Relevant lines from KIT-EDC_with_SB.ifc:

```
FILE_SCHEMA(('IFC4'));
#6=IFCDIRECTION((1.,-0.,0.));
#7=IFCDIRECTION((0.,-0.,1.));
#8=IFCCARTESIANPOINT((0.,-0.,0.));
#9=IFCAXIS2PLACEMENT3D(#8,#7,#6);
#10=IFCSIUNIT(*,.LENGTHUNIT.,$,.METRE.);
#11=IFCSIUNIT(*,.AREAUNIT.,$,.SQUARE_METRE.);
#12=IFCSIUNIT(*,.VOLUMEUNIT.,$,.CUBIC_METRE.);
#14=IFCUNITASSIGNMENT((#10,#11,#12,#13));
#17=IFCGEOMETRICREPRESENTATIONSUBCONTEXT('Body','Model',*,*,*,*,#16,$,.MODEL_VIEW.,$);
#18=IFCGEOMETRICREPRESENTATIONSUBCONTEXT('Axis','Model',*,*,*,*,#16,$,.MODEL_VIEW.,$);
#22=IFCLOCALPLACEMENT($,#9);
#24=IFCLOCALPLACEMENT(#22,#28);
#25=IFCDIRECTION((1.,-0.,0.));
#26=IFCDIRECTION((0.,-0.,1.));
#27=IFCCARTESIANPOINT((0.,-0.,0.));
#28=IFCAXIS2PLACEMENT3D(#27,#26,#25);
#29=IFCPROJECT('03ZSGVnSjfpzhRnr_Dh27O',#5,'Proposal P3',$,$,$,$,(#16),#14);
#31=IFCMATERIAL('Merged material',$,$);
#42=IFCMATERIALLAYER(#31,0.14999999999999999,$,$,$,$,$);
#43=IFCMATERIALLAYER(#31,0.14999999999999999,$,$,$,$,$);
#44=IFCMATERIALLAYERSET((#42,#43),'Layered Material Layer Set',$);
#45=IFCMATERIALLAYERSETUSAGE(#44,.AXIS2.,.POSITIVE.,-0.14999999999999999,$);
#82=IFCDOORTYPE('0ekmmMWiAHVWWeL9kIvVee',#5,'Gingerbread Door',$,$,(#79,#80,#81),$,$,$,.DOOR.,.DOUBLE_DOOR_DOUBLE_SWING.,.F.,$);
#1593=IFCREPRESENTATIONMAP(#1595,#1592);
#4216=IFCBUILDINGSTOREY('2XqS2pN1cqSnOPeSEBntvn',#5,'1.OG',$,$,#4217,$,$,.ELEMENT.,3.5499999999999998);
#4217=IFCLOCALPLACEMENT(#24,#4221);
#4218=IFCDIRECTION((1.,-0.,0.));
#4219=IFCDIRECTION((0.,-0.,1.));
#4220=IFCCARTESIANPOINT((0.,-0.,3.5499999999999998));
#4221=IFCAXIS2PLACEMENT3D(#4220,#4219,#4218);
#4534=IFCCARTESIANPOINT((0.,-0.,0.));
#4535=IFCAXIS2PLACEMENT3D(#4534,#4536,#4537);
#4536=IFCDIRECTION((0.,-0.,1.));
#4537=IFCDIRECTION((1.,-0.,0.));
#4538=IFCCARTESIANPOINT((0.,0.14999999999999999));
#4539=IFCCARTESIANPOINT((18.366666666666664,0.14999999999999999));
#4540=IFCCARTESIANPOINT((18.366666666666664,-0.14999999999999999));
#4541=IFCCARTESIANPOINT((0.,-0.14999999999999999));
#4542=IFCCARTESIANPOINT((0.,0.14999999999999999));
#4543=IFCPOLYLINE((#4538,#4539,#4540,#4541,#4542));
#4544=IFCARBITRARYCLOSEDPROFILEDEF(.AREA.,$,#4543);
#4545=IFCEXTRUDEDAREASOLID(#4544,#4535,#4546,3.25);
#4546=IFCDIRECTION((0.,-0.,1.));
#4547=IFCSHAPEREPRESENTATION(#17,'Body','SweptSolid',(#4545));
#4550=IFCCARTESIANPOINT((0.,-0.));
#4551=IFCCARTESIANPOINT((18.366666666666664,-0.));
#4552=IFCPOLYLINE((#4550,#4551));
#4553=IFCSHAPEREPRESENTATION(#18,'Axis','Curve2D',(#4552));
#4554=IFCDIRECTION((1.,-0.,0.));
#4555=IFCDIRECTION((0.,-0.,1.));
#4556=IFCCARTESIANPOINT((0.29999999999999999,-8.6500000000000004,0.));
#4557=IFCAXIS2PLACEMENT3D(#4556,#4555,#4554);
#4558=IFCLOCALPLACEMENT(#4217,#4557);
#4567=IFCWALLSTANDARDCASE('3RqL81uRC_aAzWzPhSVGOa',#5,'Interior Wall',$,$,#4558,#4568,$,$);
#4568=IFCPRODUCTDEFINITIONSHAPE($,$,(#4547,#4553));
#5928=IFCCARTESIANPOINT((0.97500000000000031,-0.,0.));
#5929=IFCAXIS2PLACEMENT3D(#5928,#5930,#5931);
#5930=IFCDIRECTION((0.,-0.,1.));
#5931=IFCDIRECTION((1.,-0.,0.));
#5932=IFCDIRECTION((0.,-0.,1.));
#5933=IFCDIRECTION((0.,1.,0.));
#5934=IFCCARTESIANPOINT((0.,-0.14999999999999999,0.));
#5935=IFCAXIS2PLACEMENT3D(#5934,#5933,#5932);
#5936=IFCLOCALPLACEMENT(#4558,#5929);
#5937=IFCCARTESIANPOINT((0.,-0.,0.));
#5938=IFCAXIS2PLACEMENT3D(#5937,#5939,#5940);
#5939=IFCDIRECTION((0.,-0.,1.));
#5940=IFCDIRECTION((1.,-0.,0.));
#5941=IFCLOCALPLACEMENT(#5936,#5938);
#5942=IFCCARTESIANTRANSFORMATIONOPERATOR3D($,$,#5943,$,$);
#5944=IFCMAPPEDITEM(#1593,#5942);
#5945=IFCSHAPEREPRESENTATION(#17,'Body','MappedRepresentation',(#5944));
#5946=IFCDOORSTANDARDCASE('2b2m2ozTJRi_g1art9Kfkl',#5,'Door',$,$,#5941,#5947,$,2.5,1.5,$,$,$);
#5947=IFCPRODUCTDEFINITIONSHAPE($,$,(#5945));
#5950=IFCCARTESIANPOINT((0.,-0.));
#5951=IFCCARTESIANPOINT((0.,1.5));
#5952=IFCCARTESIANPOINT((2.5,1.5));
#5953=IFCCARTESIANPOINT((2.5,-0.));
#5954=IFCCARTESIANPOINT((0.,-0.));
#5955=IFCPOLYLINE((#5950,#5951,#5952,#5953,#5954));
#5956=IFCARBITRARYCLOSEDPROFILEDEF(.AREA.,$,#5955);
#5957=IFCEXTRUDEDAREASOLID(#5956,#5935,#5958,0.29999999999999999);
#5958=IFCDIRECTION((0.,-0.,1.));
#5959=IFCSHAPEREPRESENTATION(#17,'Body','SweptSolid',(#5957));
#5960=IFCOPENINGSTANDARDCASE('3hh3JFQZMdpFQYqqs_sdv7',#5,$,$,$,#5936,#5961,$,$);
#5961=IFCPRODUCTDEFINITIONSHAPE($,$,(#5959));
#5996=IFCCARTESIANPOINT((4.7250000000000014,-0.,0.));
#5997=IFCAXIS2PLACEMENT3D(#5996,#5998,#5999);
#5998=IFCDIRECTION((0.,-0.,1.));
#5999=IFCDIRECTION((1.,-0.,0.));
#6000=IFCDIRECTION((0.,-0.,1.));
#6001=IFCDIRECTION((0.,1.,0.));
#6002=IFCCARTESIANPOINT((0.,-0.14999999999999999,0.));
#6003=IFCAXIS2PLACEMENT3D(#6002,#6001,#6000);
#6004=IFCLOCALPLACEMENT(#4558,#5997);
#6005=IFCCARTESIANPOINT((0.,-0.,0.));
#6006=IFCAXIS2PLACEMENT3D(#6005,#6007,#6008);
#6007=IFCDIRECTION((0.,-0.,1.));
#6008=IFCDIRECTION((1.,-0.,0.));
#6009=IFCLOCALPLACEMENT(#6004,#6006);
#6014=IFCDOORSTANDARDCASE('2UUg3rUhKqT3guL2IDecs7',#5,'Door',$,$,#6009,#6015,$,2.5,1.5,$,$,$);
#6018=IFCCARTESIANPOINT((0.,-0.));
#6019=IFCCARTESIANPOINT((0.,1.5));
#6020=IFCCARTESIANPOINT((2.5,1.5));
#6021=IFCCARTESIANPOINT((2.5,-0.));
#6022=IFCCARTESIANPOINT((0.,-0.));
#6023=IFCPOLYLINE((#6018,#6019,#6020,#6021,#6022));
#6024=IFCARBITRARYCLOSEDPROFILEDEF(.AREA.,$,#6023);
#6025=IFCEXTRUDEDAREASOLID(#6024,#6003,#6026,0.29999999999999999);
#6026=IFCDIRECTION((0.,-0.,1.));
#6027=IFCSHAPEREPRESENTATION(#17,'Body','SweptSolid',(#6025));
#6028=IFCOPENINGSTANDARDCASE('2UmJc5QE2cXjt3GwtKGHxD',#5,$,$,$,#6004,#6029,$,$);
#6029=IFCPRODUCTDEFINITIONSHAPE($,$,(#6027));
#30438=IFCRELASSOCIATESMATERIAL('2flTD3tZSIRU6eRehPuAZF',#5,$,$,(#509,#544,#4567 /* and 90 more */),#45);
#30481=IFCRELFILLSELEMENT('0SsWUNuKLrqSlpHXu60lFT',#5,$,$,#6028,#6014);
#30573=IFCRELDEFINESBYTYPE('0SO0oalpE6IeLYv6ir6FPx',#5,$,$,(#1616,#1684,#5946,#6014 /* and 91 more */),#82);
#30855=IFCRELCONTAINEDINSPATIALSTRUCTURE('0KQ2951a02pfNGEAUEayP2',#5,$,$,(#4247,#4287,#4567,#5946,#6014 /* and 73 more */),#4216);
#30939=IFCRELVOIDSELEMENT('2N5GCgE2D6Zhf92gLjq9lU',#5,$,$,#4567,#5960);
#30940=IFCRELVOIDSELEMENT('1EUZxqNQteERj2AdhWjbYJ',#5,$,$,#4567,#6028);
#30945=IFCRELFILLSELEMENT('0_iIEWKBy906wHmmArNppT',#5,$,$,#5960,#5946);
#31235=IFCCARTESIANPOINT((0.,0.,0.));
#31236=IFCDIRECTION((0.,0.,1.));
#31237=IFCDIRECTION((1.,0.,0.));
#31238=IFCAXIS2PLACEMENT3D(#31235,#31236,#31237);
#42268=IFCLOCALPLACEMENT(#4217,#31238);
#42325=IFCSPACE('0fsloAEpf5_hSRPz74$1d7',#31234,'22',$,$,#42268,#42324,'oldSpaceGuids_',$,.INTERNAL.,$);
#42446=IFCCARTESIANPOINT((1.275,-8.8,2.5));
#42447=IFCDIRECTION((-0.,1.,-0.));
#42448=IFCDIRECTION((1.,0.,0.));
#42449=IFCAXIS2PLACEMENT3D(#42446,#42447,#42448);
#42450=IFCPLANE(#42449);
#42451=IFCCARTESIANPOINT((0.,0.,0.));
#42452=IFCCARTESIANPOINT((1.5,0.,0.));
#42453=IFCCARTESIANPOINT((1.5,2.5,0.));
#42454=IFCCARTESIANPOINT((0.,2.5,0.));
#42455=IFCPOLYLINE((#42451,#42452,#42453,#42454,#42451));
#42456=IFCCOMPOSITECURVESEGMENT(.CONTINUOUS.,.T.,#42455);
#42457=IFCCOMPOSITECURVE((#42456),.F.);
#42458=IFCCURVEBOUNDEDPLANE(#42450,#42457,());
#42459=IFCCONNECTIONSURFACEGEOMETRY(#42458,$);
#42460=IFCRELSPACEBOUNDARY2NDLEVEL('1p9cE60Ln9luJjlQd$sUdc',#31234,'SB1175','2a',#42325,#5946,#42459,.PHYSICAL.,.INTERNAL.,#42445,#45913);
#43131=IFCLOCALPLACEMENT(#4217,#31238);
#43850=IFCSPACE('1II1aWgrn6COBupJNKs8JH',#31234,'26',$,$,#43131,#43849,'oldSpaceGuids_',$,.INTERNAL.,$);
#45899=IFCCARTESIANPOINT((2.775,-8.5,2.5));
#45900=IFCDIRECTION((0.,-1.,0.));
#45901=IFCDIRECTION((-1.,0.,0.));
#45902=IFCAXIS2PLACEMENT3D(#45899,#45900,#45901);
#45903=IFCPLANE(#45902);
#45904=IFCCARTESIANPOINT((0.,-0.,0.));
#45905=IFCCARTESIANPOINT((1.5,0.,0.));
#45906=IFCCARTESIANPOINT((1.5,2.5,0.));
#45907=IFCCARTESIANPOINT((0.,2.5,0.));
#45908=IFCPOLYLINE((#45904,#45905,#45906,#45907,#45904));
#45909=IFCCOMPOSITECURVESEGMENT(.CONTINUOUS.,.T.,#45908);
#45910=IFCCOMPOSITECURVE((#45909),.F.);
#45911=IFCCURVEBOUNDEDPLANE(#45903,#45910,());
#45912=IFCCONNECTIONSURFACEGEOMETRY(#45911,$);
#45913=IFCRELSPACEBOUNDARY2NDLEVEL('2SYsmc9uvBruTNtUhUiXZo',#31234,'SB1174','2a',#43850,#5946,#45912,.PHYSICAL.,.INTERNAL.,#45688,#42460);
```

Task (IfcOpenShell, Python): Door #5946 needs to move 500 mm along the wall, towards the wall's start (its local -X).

```python
import numpy as np
import ifcopenshell
import ifcopenshell.api.geometry
import ifcopenshell.util.placement
import ifcopenshell.util.unit

model = ifcopenshell.open("KIT-EDC_with_SB.ifc")
unit_scale = ifcopenshell.util.unit.calculate_unit_scale(model)

door = model.by_id(5946)
opening = door.FillsVoids[0].RelatingOpeningElement
wall = opening.VoidsElements[0].RelatingBuildingElement

wall_matrix = ifcopenshell.util.placement.get_local_placement(wall.ObjectPlacement)
shift = wall_matrix[:3, 0] * -0.5 / unit_scale
before = ifcopenshell.util.placement.get_local_placement(door.ObjectPlacement)[:3, 3].copy()

# The door is placed relative to its opening, so it follows when the opening moves.
matrix = ifcopenshell.util.placement.get_local_placement(opening.ObjectPlacement)
matrix[:3, 3] += shift
ifcopenshell.api.geometry.edit_object_placement(
    model, product=opening, matrix=matrix, is_si=False, should_transform_children=True
)

# Space boundary surfaces are stored in each space's coordinates; move them too.
for rel in door.ProvidesBoundaries:
    if not rel.ConnectionGeometry:
        continue
    surface = rel.ConnectionGeometry.SurfaceOnRelatingElement.BasisSurface
    space_matrix = ifcopenshell.util.placement.get_local_placement(rel.RelatingSpace.ObjectPlacement)
    point = np.array(surface.Position.Location.Coordinates) + space_matrix[:3, :3].T @ shift
    surface.Position = model.createIfcAxis2Placement3D(
        model.createIfcCartesianPoint(point.tolist()), surface.Position.Axis, surface.Position.RefDirection
    )

after = ifcopenshell.util.placement.get_local_placement(door.ObjectPlacement)[:3, 3]
print("door moved by", (after - before).round(3) + 0.0)

model.write("KIT-EDC_with_SB_v2.ifc")
```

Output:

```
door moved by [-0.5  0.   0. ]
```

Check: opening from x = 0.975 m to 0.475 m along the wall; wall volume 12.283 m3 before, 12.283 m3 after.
